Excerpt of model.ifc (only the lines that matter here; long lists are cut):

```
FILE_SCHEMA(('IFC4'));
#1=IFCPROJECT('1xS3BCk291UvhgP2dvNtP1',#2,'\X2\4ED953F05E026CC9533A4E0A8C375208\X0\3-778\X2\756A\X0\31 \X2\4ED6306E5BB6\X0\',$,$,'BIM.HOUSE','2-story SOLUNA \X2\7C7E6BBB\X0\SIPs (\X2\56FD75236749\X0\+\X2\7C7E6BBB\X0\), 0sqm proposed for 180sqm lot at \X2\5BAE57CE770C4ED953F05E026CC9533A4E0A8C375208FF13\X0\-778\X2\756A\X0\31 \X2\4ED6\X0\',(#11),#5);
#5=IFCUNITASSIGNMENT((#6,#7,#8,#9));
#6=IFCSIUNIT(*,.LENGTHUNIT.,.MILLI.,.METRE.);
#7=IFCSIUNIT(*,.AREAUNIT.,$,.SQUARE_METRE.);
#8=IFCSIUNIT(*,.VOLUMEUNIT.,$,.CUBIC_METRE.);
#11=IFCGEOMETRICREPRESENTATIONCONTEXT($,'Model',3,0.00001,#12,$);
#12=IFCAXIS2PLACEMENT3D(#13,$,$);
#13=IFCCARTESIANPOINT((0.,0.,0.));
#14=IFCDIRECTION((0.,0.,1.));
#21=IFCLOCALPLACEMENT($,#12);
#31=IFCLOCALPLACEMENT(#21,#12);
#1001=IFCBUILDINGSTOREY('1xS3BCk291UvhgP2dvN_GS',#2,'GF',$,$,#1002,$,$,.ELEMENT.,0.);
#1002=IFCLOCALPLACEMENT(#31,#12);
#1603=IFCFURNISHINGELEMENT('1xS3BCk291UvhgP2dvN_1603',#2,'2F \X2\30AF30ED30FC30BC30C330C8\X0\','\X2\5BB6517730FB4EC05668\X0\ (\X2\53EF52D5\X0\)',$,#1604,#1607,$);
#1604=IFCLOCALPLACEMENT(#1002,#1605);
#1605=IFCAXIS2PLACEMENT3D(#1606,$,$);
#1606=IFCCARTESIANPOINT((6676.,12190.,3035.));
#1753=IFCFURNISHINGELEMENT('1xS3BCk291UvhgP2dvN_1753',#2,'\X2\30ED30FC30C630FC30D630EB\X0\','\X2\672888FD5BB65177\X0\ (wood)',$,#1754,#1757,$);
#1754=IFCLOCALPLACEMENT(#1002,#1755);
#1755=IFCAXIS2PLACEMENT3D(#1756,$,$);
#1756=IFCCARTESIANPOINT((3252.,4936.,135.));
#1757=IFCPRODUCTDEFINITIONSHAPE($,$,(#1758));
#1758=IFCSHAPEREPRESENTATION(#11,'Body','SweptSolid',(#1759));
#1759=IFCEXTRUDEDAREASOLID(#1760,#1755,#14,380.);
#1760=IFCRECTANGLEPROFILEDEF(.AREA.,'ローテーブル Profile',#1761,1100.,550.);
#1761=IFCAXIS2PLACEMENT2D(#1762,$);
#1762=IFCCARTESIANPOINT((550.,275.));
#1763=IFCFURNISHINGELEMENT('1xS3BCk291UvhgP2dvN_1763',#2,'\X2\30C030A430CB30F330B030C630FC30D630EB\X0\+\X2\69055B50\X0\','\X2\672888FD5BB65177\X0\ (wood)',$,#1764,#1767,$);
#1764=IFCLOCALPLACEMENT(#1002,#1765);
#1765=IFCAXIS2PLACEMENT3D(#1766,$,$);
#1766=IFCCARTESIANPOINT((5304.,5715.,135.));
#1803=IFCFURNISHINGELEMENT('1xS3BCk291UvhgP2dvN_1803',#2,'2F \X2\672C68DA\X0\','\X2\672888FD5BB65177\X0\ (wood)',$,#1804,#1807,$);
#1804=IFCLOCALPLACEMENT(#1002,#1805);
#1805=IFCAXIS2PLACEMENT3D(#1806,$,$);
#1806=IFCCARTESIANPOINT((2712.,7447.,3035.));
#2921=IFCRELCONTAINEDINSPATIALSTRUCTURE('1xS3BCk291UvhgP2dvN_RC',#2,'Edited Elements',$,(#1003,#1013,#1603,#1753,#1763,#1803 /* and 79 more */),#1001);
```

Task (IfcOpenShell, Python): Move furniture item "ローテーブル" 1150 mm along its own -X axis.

```python
import ifcopenshell
import ifcopenshell.api.geometry
import ifcopenshell.util.placement
import ifcopenshell.util.unit

model = ifcopenshell.open("model.ifc")
unit_scale = ifcopenshell.util.unit.calculate_unit_scale(model)

item = model.by_guid("1xS3BCk291UvhgP2dvN_1753")
matrix = ifcopenshell.util.placement.get_local_placement(item.ObjectPlacement)
matrix[:3, 3] -= matrix[:3, 0] * 1.15 / unit_scale
ifcopenshell.api.geometry.edit_object_placement(model, product=item, matrix=matrix, is_si=False)

print(ifcopenshell.util.placement.get_local_placement(item.ObjectPlacement).round(3) + 0.0)

model.write("model_rev.ifc")
```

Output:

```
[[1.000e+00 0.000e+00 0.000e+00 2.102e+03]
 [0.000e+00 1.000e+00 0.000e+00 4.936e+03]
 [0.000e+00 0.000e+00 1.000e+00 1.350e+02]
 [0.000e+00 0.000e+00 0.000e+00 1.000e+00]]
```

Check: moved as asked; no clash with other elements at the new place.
